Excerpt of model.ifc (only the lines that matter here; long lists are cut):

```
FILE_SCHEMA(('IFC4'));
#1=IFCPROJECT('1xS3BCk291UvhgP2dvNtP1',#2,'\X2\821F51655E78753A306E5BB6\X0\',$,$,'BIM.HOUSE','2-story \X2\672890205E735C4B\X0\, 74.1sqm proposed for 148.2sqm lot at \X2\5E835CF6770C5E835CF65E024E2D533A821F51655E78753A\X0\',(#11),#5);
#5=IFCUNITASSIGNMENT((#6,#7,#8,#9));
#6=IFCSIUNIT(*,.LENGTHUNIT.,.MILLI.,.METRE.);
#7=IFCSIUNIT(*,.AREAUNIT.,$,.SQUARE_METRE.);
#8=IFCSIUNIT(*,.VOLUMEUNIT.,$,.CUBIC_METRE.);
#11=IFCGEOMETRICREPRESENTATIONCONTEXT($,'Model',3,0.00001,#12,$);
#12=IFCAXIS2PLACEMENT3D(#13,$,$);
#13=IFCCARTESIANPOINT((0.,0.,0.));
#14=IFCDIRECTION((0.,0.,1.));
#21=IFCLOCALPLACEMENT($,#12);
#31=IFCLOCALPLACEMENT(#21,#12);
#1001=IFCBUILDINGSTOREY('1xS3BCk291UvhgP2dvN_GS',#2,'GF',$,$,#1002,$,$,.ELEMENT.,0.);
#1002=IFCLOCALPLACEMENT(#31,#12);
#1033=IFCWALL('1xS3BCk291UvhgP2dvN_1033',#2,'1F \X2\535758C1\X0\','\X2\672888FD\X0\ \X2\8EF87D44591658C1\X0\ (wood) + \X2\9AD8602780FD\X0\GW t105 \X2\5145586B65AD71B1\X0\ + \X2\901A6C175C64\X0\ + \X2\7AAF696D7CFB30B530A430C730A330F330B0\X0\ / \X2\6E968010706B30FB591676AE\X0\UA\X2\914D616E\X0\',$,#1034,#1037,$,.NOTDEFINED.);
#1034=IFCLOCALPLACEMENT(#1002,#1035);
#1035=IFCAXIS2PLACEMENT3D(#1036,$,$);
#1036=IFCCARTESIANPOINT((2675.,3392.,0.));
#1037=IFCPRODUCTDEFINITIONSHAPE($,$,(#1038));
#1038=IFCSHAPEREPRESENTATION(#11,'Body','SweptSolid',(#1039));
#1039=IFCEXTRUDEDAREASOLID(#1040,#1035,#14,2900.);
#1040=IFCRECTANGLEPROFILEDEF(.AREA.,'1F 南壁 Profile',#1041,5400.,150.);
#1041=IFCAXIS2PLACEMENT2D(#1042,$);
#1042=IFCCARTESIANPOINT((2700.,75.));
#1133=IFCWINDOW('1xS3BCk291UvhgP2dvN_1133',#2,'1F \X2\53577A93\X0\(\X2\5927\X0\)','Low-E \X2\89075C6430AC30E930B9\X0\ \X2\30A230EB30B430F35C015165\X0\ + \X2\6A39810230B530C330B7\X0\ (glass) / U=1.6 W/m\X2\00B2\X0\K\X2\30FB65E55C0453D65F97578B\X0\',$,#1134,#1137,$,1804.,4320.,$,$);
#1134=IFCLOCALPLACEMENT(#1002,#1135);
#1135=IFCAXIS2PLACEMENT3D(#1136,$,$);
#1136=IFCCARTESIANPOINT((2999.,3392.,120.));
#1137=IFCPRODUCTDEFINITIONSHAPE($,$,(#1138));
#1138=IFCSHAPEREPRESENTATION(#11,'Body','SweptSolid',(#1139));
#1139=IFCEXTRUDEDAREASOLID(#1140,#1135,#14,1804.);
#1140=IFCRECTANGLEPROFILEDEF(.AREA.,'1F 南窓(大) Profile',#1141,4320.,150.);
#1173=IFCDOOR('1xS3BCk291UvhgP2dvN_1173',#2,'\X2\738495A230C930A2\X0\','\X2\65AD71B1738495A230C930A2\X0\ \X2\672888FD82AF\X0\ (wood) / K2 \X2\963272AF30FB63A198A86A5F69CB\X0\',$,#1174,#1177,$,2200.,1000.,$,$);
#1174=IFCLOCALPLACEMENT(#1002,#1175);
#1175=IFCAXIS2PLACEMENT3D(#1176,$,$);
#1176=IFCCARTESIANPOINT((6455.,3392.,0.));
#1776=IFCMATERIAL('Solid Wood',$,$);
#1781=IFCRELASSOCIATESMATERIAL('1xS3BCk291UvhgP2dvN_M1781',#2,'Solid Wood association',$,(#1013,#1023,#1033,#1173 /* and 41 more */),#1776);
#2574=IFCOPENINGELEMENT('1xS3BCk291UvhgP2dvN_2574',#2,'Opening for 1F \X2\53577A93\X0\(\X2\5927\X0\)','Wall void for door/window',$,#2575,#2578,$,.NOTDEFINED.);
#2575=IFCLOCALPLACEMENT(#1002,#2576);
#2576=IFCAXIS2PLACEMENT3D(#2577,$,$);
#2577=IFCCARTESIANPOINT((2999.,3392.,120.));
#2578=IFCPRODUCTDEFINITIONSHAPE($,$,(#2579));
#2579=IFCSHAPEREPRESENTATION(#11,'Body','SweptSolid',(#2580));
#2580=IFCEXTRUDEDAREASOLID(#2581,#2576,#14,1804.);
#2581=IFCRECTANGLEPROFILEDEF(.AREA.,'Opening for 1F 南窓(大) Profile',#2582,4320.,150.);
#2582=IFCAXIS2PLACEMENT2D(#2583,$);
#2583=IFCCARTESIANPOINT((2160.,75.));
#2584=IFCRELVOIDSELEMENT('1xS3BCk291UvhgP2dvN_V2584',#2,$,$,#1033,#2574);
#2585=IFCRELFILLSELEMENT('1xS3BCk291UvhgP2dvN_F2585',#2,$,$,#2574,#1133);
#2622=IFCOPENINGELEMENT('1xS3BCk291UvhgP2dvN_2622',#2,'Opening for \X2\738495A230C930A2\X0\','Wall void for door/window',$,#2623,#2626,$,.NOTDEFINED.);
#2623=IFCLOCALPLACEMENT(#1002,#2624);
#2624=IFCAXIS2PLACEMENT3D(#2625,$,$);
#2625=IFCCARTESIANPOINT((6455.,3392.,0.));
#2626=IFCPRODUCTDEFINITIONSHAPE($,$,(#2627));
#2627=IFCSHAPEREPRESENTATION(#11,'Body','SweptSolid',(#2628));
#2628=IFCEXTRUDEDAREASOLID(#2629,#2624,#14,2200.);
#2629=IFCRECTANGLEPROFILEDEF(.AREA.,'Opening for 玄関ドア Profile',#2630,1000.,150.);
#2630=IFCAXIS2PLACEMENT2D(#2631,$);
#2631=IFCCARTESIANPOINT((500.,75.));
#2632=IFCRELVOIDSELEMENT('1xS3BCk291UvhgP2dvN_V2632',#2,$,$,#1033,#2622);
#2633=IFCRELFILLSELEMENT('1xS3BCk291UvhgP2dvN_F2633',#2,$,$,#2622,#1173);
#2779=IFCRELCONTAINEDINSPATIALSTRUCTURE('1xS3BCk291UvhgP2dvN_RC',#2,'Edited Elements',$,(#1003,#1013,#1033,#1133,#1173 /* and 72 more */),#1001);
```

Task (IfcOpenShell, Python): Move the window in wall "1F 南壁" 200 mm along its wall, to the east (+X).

```python
import ifcopenshell
import ifcopenshell.api.geometry
import ifcopenshell.util.placement
import ifcopenshell.util.unit

model = ifcopenshell.open("model.ifc")
unit_scale = ifcopenshell.util.unit.calculate_unit_scale(model)

window = model.by_id(1133)
opening = window.FillsVoids[0].RelatingOpeningElement
wall = opening.VoidsElements[0].RelatingBuildingElement

wall_matrix = ifcopenshell.util.placement.get_local_placement(wall.ObjectPlacement)
shift = wall_matrix[:3, 0] * 0.2 / unit_scale
before = ifcopenshell.util.placement.get_local_placement(window.ObjectPlacement)[:3, 3].copy()

# The window is not placed relative to its opening, so move both.
for product in (opening, window):
    matrix = ifcopenshell.util.placement.get_local_placement(product.ObjectPlacement)
    matrix[:3, 3] += shift
    ifcopenshell.api.geometry.edit_object_placement(model, product=product, matrix=matrix, is_si=False)

after = ifcopenshell.util.placement.get_local_placement(window.ObjectPlacement)[:3, 3]
print("window moved by", (after - before).round(3) + 0.0)

model.write("model-out.ifc")
```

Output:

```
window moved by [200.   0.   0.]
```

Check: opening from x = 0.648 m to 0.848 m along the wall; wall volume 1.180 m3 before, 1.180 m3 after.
